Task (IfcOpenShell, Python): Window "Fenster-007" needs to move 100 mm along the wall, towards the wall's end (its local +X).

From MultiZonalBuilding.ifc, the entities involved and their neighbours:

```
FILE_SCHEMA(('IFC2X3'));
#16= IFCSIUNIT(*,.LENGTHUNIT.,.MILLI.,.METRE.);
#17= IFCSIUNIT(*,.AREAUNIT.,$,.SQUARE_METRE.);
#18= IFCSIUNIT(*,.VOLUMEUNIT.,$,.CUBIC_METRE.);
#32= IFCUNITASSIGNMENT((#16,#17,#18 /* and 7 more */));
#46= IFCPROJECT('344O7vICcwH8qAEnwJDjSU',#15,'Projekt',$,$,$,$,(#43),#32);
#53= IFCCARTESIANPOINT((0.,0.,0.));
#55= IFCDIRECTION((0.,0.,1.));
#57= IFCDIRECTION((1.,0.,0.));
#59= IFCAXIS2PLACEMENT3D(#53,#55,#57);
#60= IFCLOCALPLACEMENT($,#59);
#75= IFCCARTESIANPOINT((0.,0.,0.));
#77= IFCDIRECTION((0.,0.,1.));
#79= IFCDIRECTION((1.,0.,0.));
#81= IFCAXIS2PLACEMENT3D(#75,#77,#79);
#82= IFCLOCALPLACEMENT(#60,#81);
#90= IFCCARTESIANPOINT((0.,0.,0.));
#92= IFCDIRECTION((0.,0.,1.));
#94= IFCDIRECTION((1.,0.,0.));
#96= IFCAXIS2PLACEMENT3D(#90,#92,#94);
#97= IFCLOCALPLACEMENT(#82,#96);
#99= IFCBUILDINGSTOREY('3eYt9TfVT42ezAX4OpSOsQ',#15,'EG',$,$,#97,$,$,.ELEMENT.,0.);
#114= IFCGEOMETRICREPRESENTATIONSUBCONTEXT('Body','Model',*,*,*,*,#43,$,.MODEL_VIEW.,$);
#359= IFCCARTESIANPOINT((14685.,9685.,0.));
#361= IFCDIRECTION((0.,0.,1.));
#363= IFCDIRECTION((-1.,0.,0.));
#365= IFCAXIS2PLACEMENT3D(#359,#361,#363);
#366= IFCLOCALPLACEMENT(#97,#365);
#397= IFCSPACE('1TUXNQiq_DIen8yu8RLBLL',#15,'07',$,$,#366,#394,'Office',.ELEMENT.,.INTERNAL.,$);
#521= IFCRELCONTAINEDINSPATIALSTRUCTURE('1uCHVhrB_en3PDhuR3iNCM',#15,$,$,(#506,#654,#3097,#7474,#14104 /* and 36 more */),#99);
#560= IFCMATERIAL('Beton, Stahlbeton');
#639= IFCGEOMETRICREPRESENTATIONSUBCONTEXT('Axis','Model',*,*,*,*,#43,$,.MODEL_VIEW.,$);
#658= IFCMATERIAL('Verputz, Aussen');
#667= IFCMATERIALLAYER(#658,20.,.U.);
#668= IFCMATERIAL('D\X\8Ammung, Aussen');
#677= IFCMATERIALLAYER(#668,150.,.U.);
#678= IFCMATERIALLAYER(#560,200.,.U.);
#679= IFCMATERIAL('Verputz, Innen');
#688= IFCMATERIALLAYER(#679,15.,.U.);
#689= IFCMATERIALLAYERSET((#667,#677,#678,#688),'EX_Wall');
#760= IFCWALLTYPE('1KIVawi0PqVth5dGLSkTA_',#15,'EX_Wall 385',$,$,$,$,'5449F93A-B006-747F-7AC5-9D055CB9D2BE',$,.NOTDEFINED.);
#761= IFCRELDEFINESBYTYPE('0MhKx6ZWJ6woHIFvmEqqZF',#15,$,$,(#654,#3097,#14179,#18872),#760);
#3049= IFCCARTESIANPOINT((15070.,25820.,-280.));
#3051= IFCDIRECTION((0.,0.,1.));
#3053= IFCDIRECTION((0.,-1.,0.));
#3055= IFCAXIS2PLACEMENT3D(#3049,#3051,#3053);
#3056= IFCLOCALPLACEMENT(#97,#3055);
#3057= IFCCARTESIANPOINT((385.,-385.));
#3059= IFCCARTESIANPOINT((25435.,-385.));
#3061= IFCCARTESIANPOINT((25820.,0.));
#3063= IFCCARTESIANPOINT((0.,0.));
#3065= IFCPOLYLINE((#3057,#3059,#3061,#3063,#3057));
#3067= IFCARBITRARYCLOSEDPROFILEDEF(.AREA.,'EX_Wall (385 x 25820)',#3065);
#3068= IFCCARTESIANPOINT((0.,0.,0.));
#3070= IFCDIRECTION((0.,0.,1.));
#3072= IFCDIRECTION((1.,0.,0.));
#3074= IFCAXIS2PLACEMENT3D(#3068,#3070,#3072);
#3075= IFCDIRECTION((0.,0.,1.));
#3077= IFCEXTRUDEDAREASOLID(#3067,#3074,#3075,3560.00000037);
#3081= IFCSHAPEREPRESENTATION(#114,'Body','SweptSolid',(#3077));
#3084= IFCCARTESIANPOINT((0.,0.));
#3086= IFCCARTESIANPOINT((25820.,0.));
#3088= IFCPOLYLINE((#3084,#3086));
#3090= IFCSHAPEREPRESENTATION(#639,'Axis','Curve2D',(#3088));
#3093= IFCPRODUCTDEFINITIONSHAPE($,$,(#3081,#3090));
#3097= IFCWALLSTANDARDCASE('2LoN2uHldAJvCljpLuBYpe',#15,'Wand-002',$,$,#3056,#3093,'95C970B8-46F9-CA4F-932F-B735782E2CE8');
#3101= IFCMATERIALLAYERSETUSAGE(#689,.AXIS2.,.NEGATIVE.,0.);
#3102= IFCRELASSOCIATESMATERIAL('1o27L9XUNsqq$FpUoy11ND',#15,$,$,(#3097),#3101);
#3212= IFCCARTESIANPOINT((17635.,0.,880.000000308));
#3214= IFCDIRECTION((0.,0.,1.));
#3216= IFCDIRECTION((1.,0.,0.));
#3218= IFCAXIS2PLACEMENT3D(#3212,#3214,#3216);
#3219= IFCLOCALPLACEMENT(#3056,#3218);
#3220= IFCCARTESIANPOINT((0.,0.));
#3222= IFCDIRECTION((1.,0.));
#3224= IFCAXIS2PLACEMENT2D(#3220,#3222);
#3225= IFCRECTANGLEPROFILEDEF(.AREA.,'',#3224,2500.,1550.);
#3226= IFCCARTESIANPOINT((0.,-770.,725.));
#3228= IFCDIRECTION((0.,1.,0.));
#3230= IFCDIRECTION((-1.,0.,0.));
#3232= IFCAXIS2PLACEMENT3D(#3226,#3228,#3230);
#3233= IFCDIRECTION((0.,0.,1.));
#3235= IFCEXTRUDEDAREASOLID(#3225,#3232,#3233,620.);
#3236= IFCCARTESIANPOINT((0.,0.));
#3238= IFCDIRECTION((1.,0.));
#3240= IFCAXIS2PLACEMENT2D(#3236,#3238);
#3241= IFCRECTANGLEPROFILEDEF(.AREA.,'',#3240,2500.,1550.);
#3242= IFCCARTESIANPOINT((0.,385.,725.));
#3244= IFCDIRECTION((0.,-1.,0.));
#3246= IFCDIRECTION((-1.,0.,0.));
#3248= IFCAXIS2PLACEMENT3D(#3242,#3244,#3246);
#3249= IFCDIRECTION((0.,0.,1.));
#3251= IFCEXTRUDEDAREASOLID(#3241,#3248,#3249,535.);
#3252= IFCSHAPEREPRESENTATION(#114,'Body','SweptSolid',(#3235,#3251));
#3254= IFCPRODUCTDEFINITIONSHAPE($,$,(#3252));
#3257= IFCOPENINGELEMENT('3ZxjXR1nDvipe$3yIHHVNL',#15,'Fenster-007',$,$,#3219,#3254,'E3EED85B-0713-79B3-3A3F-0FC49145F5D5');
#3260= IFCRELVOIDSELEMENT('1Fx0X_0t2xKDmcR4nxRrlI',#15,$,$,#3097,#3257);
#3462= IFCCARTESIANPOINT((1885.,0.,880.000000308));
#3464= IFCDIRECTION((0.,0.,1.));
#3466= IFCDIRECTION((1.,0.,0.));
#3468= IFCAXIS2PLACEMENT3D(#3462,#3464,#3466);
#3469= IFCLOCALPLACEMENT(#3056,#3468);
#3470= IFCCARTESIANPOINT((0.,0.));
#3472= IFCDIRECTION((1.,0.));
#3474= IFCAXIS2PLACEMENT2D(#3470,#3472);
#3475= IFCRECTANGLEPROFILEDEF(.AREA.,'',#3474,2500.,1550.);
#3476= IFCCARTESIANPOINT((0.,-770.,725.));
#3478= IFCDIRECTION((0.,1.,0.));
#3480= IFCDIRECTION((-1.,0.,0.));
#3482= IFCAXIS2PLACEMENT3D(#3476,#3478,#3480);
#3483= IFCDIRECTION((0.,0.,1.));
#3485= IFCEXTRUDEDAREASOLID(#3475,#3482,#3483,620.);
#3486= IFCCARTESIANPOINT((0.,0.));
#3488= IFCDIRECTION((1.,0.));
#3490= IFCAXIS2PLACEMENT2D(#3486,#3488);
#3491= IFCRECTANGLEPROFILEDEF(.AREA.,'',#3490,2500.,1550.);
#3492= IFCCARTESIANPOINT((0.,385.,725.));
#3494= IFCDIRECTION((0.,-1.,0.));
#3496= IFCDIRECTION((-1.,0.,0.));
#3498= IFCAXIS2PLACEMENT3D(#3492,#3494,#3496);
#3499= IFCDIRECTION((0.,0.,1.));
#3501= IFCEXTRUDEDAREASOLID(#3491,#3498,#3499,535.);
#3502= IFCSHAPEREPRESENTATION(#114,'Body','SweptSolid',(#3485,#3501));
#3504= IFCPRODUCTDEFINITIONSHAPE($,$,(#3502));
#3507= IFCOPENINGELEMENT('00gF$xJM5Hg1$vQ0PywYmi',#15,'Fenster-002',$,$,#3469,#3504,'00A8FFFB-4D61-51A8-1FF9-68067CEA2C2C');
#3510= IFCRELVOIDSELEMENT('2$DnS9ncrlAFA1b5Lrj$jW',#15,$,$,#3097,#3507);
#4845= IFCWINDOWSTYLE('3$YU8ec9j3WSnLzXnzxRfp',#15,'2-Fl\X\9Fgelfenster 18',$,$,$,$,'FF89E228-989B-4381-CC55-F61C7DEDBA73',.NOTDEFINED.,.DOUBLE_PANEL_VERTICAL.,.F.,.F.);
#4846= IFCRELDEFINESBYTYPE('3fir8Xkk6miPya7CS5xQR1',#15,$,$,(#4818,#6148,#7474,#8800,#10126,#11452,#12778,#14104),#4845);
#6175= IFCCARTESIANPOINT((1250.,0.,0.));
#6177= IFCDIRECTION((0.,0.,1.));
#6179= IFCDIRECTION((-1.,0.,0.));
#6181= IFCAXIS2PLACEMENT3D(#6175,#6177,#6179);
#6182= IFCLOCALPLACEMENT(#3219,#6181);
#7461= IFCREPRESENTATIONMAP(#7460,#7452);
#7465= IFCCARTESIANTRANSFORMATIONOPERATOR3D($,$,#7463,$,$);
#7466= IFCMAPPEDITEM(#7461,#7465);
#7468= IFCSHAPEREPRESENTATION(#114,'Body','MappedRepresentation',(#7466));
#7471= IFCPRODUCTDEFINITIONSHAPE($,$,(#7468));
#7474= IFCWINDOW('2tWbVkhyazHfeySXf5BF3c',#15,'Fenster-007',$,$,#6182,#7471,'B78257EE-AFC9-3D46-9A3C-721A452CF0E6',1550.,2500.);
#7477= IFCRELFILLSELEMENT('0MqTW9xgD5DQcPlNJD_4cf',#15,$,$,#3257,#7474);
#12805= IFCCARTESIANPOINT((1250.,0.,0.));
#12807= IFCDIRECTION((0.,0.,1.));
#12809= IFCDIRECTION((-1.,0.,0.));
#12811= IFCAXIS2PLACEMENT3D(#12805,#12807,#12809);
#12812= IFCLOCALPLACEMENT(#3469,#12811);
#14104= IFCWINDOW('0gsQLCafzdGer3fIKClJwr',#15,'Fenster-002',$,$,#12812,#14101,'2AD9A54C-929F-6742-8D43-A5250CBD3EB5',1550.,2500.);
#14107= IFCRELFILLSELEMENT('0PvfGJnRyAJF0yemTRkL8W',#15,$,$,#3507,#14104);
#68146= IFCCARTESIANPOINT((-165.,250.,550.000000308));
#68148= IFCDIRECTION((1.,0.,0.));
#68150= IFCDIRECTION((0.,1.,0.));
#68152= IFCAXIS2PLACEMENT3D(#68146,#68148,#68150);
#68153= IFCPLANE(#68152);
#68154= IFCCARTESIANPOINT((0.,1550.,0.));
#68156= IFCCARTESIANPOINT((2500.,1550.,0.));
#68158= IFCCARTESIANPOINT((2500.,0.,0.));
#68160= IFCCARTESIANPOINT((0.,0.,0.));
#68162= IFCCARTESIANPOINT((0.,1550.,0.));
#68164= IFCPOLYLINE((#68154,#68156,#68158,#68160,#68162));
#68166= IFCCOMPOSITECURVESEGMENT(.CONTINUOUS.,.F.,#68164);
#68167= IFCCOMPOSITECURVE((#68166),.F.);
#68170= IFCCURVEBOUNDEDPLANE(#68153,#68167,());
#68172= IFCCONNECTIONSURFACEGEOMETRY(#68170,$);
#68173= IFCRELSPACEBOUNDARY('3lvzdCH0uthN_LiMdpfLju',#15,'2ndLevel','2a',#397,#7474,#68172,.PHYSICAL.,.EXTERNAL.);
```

```python
import numpy as np
import ifcopenshell
import ifcopenshell.api.geometry
import ifcopenshell.util.placement
import ifcopenshell.util.unit

model = ifcopenshell.open("MultiZonalBuilding.ifc")
unit_scale = ifcopenshell.util.unit.calculate_unit_scale(model)

window = model.by_guid("2tWbVkhyazHfeySXf5BF3c")
opening = window.FillsVoids[0].RelatingOpeningElement
wall = opening.VoidsElements[0].RelatingBuildingElement

wall_matrix = ifcopenshell.util.placement.get_local_placement(wall.ObjectPlacement)
shift = wall_matrix[:3, 0] * 0.1 / unit_scale
before = ifcopenshell.util.placement.get_local_placement(window.ObjectPlacement)[:3, 3].copy()

# The window is placed relative to its opening, so it follows when the opening moves.
matrix = ifcopenshell.util.placement.get_local_placement(opening.ObjectPlacement)
matrix[:3, 3] += shift
ifcopenshell.api.geometry.edit_object_placement(
    model, product=opening, matrix=matrix, is_si=False, should_transform_children=True
)

# Space boundary surfaces are stored in each space's coordinates; move them too.
for rel in window.ProvidesBoundaries:
    if not rel.ConnectionGeometry:
        continue
    surface = rel.ConnectionGeometry.SurfaceOnRelatingElement.BasisSurface
    space_matrix = ifcopenshell.util.placement.get_local_placement(rel.RelatingSpace.ObjectPlacement)
    point = np.array(surface.Position.Location.Coordinates) + space_matrix[:3, :3].T @ shift
    surface.Position = model.createIfcAxis2Placement3D(
        model.createIfcCartesianPoint(point.tolist()), surface.Position.Axis, surface.Position.RefDirection
    )

after = ifcopenshell.util.placement.get_local_placement(window.ObjectPlacement)[:3, 3]
print("window moved by", (after - before).round(3) + 0.0)

model.write("MultiZonalBuilding_edited.ifc")
```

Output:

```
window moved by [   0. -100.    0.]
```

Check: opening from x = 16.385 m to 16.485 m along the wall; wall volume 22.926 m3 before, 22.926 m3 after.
